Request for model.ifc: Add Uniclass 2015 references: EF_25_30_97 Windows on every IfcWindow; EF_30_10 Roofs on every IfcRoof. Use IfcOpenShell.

First a look at what the model holds.

```python
import ifcopenshell

model = ifcopenshell.open("model.ifc")
print(model.schema)
print("classifications:", [c.Name for c in model.by_type("IfcClassification")])
for ifc_class in ("IfcDoor", "IfcRoof", "IfcStair", "IfcWall", "IfcWindow"):
    print(ifc_class, len(model.by_type(ifc_class)))
```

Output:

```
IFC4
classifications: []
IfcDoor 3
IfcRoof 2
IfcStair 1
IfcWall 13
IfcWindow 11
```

```python
import ifcopenshell
import ifcopenshell.api.classification

model = ifcopenshell.open("model.ifc")

system = ifcopenshell.api.classification.add_classification(model, classification="Uniclass 2015")

codes = {
    "IfcWindow": ("EF_25_30_97", "Windows"),
    "IfcRoof": ("EF_30_10", "Roofs"),
}
for ifc_class, (code, name) in codes.items():
    products = model.by_type(ifc_class)
    ifcopenshell.api.classification.add_reference(
        model, products=products, classification=system, identification=code, name=name
    )
    print(code, len(products))

model.write("model_edited.ifc")
```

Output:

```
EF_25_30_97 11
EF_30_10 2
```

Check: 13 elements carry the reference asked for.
